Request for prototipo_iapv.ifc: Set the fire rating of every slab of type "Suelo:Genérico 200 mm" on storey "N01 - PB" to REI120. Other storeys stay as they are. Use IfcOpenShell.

First a look at what the model holds.

```python
import ifcopenshell
import ifcopenshell.util.element

model = ifcopenshell.open("prototipo_iapv.ifc")
print(model.schema)
storey = next(s for s in model.by_type("IfcBuildingStorey") if s.Name == "N01 - PB")
slabs = [e for e in ifcopenshell.util.element.get_decomposition(storey) if e.is_a("IfcSlab")]
seen = {}
for e in slabs:
    element_type = ifcopenshell.util.element.get_type(e)
    key = (element_type.Name if element_type != e and element_type else None, ifcopenshell.util.element.get_pset(e, "Pset_SlabCommon", "FireRating"))
    seen[key] = seen.get(key, 0) + 1
for (name, value), count in sorted(seen.items(), key=str):
    print(count, "x", name, "|", value)
```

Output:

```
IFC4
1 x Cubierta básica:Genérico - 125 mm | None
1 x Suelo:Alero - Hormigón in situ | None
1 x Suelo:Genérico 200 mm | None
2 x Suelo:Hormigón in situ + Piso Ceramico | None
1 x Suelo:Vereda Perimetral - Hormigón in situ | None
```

```python
import ifcopenshell
import ifcopenshell.api.pset
import ifcopenshell.util.element

model = ifcopenshell.open("prototipo_iapv.ifc")

storey = next(s for s in model.by_type("IfcBuildingStorey") if s.Name == "N01 - PB")
slabs = [e for e in ifcopenshell.util.element.get_decomposition(storey) if e.is_a("IfcSlab")]

count = 0
for e in slabs:
    element_type = ifcopenshell.util.element.get_type(e)
    if element_type in (None, e) or element_type.Name != "Suelo:Genérico 200 mm":
        continue
    # add_pset returns the element's existing set when there is one.
    pset = ifcopenshell.api.pset.add_pset(model, product=e, name="Pset_SlabCommon")
    ifcopenshell.api.pset.edit_pset(model, pset=pset, properties={"FireRating": "REI120"})
    count += 1

print(count, "slabs updated")

model.write("prototipo_iapv-out.ifc")
```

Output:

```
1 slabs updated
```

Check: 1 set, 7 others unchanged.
